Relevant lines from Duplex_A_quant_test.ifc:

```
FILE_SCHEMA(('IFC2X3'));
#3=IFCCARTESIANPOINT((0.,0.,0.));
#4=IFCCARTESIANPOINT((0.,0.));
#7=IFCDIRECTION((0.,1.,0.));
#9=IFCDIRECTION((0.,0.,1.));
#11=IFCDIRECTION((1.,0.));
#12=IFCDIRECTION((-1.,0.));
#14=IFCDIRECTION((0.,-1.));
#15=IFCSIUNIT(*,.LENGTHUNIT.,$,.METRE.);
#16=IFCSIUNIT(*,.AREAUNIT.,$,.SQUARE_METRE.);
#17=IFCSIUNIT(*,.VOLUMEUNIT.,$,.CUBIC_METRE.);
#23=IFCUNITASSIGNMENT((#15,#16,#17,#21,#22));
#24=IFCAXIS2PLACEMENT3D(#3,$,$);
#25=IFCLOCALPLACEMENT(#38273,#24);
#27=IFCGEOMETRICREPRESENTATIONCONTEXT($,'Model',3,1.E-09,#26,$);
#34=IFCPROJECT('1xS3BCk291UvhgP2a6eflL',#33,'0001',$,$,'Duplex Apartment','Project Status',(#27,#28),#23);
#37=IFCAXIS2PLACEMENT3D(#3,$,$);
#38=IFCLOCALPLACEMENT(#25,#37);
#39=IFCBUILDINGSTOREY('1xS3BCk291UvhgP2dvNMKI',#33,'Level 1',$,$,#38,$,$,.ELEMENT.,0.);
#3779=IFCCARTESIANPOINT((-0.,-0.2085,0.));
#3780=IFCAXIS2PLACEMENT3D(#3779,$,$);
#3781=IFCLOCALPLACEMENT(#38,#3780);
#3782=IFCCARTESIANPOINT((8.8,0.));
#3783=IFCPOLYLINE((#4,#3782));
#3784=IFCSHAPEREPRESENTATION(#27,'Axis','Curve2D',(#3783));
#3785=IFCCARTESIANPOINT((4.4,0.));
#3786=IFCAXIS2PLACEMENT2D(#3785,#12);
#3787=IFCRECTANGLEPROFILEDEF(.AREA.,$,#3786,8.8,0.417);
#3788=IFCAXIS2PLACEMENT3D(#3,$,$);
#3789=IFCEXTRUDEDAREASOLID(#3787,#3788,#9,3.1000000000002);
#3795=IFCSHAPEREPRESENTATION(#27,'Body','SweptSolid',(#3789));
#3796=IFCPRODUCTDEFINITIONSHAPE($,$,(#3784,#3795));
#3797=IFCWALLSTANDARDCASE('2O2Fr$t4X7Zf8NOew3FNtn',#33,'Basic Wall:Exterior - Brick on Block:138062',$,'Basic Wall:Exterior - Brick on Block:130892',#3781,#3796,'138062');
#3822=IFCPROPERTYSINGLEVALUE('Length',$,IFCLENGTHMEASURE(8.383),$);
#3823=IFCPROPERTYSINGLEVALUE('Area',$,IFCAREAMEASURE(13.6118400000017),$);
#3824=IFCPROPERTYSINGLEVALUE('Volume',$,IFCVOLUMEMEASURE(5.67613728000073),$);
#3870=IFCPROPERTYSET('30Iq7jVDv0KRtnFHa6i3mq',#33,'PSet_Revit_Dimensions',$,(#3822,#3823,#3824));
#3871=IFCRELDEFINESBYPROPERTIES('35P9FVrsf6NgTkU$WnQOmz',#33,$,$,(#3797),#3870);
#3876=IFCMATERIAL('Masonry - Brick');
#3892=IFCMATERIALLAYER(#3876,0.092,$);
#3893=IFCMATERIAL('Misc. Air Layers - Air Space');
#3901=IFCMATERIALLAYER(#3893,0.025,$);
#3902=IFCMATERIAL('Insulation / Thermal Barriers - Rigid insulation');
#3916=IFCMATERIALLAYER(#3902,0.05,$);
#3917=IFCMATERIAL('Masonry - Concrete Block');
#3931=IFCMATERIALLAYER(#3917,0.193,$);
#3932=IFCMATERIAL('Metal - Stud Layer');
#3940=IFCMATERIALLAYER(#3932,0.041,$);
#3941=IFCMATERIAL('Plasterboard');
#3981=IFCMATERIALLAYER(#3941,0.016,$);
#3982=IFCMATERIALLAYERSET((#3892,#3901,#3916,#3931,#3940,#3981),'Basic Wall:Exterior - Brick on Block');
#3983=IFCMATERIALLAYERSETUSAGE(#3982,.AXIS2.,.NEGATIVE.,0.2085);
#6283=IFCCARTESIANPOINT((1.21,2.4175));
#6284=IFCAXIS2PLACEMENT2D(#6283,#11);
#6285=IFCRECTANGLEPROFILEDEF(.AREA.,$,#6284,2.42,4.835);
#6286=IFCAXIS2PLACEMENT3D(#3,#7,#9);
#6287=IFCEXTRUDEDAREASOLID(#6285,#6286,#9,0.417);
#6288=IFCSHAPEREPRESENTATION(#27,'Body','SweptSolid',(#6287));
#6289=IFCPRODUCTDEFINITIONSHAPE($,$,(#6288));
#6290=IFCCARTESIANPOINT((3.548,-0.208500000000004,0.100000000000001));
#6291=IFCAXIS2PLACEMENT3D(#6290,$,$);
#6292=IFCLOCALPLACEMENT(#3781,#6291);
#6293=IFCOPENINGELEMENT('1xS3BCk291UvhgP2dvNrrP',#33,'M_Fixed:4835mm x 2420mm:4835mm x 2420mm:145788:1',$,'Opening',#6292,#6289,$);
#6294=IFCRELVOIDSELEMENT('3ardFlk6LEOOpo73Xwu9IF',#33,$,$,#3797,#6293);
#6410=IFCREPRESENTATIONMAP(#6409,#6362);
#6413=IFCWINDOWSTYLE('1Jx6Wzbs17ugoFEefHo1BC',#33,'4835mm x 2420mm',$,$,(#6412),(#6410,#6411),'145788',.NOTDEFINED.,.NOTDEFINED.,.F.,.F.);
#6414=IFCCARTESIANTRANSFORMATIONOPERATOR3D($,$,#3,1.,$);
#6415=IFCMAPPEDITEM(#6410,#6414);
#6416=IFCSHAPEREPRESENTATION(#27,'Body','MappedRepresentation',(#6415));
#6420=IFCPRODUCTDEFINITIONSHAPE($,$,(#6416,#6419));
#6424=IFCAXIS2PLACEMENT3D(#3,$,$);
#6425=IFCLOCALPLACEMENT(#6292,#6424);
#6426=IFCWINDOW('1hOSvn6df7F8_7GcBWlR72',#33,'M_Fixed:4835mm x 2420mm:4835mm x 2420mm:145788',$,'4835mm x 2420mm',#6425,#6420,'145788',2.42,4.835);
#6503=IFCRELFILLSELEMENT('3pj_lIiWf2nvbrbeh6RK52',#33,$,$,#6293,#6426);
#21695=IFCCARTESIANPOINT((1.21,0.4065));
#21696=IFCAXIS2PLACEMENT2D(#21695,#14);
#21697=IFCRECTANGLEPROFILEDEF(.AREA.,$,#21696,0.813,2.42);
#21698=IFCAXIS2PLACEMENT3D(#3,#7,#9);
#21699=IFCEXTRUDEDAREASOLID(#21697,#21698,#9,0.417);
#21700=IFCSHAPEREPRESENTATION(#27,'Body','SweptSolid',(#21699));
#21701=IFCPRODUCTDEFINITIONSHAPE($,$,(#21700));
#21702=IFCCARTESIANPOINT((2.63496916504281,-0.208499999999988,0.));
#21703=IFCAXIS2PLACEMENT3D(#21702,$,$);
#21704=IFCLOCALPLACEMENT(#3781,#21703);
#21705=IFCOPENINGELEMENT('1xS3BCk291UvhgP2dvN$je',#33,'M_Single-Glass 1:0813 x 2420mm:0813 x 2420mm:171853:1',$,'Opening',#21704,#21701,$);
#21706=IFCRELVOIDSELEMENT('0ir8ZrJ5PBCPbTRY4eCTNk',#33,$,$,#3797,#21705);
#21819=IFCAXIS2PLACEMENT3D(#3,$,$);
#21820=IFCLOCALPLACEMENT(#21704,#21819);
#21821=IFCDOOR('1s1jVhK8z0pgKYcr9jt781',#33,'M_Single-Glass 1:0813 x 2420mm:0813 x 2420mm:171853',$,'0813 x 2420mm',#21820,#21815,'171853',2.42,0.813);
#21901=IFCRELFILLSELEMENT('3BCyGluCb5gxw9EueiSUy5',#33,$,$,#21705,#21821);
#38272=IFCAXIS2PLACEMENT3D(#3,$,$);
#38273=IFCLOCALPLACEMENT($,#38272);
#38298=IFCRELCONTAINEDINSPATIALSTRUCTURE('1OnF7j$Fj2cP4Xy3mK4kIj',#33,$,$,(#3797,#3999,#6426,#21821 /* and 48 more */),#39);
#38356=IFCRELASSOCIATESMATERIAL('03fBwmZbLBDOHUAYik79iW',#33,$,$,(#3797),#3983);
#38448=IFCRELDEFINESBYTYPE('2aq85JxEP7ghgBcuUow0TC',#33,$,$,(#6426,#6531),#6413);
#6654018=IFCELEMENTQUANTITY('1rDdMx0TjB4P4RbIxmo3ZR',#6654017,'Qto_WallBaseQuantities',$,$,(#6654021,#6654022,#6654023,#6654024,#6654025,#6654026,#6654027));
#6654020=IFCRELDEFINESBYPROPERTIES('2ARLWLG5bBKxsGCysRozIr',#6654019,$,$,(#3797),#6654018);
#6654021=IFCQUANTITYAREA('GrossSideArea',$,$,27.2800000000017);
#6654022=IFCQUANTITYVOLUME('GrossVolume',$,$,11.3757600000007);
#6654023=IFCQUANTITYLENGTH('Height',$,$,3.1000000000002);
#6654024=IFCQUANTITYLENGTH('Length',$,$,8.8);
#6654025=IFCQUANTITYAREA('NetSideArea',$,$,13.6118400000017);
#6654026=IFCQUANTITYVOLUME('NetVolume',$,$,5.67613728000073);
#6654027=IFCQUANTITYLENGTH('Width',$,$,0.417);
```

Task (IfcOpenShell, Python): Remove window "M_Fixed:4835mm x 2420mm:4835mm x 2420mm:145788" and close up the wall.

```python
import ifcopenshell
import ifcopenshell.api.feature
import ifcopenshell.api.pset
import ifcopenshell.api.root
import ifcopenshell.geom
import ifcopenshell.util.element
import ifcopenshell.util.shape
import ifcopenshell.util.unit

model = ifcopenshell.open("Duplex_A_quant_test.ifc")
area_scale = ifcopenshell.util.unit.calculate_unit_scale(model, "AREAUNIT")
volume_scale = ifcopenshell.util.unit.calculate_unit_scale(model, "VOLUMEUNIT")
settings = ifcopenshell.geom.settings()


def volume(element):
    """Net volume in cubic metres, openings subtracted."""
    shape = ifcopenshell.geom.create_shape(settings, element)
    return ifcopenshell.util.shape.get_volume(shape.geometry)


window = model.by_guid("1hOSvn6df7F8_7GcBWlR72")
opening = window.FillsVoids[0].RelatingOpeningElement
wall = opening.VoidsElements[0].RelatingBuildingElement
before = volume(wall)

ifcopenshell.api.root.remove_product(model, product=window)
ifcopenshell.api.feature.remove_feature(model, feature=opening)

after = volume(wall)
thickness = 0.417  # wall thickness in metres

# Update the wall's stored quantities.
pset = model.by_id(ifcopenshell.util.element.get_pset(wall, "PSet_Revit_Dimensions", should_inherit=False)["id"])
ifcopenshell.api.pset.edit_pset(model, pset=pset, properties={
    "Area": model.create_entity("IfcAreaMeasure", after / thickness / area_scale),
    "Volume": model.create_entity("IfcVolumeMeasure", after / volume_scale),
})
qto = model.by_id(ifcopenshell.util.element.get_pset(wall, "Qto_WallBaseQuantities", should_inherit=False)["id"])
ifcopenshell.api.pset.edit_qto(model, qto=qto, properties={
    "NetSideArea": after / thickness / area_scale,
    "NetVolume": after / volume_scale,
})

print(f"wall volume {before:.3f} -> {after:.3f} m3")

model.write("Duplex_A_quant_test_v2.ifc")
```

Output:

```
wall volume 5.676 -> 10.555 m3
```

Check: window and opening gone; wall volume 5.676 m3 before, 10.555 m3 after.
